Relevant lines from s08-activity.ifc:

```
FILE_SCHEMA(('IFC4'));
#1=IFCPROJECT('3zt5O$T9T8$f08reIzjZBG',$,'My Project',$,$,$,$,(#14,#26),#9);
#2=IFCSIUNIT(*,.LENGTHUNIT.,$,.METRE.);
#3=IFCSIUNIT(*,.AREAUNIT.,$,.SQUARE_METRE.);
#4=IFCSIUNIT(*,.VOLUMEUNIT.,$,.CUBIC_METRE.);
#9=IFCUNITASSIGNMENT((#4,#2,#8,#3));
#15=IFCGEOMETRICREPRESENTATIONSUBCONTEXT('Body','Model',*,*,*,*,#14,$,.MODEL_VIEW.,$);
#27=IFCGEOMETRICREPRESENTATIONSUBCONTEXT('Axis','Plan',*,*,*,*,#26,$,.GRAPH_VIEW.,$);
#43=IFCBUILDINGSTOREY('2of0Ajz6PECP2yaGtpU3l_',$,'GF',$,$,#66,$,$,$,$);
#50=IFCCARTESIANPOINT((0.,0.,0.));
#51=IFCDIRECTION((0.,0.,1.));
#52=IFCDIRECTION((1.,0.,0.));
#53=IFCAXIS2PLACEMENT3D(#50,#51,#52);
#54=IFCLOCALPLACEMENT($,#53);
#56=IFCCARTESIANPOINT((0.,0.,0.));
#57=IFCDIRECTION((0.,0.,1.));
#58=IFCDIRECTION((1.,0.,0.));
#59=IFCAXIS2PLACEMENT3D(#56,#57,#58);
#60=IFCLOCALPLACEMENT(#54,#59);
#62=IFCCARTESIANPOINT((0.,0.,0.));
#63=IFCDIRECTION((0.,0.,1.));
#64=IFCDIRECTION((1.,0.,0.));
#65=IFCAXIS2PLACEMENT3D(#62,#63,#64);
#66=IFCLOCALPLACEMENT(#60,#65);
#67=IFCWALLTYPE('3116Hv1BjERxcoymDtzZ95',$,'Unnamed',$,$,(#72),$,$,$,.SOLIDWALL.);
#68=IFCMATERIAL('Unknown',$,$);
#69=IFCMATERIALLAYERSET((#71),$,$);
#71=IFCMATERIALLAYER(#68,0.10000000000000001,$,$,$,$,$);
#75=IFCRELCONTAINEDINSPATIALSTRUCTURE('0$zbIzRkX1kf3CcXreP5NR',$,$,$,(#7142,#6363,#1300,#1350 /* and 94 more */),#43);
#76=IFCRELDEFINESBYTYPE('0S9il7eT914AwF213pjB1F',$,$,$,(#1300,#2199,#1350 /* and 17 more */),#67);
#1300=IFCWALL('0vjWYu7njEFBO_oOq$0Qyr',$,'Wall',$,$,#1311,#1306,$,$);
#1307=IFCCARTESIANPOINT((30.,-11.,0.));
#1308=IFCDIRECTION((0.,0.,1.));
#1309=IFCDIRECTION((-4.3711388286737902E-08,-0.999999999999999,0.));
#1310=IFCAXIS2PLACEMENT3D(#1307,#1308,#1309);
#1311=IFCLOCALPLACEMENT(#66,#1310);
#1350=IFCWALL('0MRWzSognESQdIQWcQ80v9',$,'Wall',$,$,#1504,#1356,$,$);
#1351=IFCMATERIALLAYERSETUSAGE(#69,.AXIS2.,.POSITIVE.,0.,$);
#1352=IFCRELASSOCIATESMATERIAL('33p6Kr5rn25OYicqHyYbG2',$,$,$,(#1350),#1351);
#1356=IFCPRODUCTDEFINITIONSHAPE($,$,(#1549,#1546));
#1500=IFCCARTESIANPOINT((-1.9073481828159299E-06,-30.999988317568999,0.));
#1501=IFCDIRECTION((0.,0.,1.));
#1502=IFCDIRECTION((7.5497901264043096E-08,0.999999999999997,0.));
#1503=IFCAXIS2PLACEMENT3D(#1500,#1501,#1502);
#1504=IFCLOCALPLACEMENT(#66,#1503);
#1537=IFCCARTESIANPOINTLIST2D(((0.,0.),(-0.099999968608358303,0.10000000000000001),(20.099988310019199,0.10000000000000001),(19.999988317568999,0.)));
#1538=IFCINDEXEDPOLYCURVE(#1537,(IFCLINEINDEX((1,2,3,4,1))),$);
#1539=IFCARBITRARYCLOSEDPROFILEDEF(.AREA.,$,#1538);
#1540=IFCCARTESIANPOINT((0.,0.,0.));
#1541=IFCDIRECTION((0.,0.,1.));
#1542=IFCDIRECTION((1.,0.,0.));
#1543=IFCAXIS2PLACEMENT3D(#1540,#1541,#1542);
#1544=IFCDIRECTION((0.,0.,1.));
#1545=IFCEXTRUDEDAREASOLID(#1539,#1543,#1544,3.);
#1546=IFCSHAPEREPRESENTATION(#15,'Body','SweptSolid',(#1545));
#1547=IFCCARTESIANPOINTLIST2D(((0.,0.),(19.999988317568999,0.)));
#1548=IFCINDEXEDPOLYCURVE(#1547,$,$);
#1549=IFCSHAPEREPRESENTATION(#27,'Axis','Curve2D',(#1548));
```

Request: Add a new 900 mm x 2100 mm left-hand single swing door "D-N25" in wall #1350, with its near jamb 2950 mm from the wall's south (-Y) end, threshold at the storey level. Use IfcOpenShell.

```python
import numpy as np
import ifcopenshell
import ifcopenshell.api.feature
import ifcopenshell.api.geometry
import ifcopenshell.api.root
import ifcopenshell.api.spatial
import ifcopenshell.geom
import ifcopenshell.util.element
import ifcopenshell.util.placement
import ifcopenshell.util.representation
import ifcopenshell.util.shape
import ifcopenshell.util.unit

model = ifcopenshell.open("s08-activity.ifc")
unit_scale = ifcopenshell.util.unit.calculate_unit_scale(model)
settings = ifcopenshell.geom.settings()


def volume(element):
    """Net volume in cubic metres, openings subtracted."""
    shape = ifcopenshell.geom.create_shape(settings, element)
    return ifcopenshell.util.shape.get_volume(shape.geometry)


wall = model.by_guid("0MRWzSognESQdIQWcQ80v9")
storey = ifcopenshell.util.element.get_container(wall, ifc_class="IfcBuildingStorey")
context = ifcopenshell.util.representation.get_context(model, "Model", "Body", "MODEL_VIEW")
before = volume(wall)

width, height, from_end, sill = 0.9, 2.1, 2.95, 0.0  # metres

# The wall runs along its own X axis, and the end named is its -X end.
wall_shape = ifcopenshell.geom.create_shape(settings, wall)
x, y, z = ifcopenshell.util.shape.get_vertices(wall_shape.geometry).T
start = x.min() + from_end
face, thickness = float(y.min()), float(y.max() - y.min())
wall_matrix = ifcopenshell.util.placement.get_local_placement(wall.ObjectPlacement)
level = ifcopenshell.util.placement.get_local_placement(storey.ObjectPlacement)[2, 3]


def in_wall(x, y):
    """Placement at x, y metres in the wall's axes, at sill height."""
    matrix = wall_matrix.copy()
    matrix[:, 3] = wall_matrix @ np.array([x / unit_scale, y / unit_scale, 0.0, 1.0])
    matrix[2, 3] = level + sill / unit_scale
    return matrix


# Opening: a box that overshoots both wall faces by 50 mm.
opening = ifcopenshell.api.root.create_entity(model, ifc_class="IfcOpeningElement", predefined_type="OPENING")
box = ifcopenshell.api.geometry.add_wall_representation(
    model, context=context, length=width, height=height, thickness=thickness + 0.1
)
ifcopenshell.api.geometry.assign_representation(model, product=opening, representation=box)
ifcopenshell.api.geometry.edit_object_placement(model, product=opening, matrix=in_wall(start, face - 0.05), is_si=False)
ifcopenshell.api.feature.add_feature(model, feature=opening, element=wall)

door = ifcopenshell.api.root.create_entity(model, ifc_class="IfcDoor", name="D-N25", predefined_type="DOOR")
door.OverallWidth, door.OverallHeight = width / unit_scale, height / unit_scale
door.OperationType = "SINGLE_SWING_LEFT"
body = ifcopenshell.api.geometry.add_door_representation(
    model,
    context=context,
    overall_width=door.OverallWidth,
    overall_height=door.OverallHeight,
    operation_type="SINGLE_SWING_LEFT",
    lining_properties={"LiningDepth": thickness / unit_scale, "ThresholdDepth": thickness / unit_scale},
)
ifcopenshell.api.geometry.assign_representation(model, product=door, representation=body)
ifcopenshell.api.spatial.assign_container(model, products=[door], relating_structure=storey)
ifcopenshell.api.feature.add_filling(model, opening=opening, element=door)

# The lining spans the wall, so the door starts at the wall face.
ifcopenshell.api.geometry.edit_object_placement(model, product=door, matrix=in_wall(start, face), is_si=False)

after = volume(wall)

print(f"wall volume {before:.3f} -> {after:.3f} m3")

model.write("s08-activity_updated.ifc")
```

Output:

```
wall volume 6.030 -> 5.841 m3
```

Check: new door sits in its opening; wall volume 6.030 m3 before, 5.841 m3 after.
